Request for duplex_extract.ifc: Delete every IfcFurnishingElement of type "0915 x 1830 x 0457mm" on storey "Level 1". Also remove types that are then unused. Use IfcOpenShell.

First a look at what the model holds.

```python
import ifcopenshell
import ifcopenshell.util.element

model = ifcopenshell.open("duplex_extract.ifc")
print(model.schema)
storey = next(s for s in model.by_type("IfcBuildingStorey") if s.Name == "Level 1")
furniture = [e for e in ifcopenshell.util.element.get_decomposition(storey) if e.is_a("IfcFurnishingElement")]
seen = {}
for e in furniture:
    element_type = ifcopenshell.util.element.get_type(e)
    name = element_type.Name if element_type not in (None, e) else None
    seen[name] = seen.get(name, 0) + 1
for name, count in sorted(seen.items(), key=str):
    print(count, "x", name)
```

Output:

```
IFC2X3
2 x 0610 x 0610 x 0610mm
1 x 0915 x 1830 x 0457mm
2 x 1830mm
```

```python
import ifcopenshell
import ifcopenshell.api.root
import ifcopenshell.util.element

model = ifcopenshell.open("duplex_extract.ifc")

storey = next(s for s in model.by_type("IfcBuildingStorey") if s.Name == "Level 1")
furniture = [e for e in ifcopenshell.util.element.get_decomposition(storey) if e.is_a("IfcFurnishingElement")]
targets = [e for e in furniture if (t := ifcopenshell.util.element.get_type(e)) not in (None, e) and t.Name == "0915 x 1830 x 0457mm"]
types = {ifcopenshell.util.element.get_type(e) for e in targets} - {None, *targets}

for e in targets:
    ifcopenshell.api.root.remove_product(model, product=e)
print(len(targets), "removed")

unused = [t for t in types if not ifcopenshell.util.element.get_types(t)]
for t in unused:
    ifcopenshell.api.root.remove_product(model, product=t)
print(len(unused), "unused types removed")

model.write("duplex_extract_rev.ifc")
```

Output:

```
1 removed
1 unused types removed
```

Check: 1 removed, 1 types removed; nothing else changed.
